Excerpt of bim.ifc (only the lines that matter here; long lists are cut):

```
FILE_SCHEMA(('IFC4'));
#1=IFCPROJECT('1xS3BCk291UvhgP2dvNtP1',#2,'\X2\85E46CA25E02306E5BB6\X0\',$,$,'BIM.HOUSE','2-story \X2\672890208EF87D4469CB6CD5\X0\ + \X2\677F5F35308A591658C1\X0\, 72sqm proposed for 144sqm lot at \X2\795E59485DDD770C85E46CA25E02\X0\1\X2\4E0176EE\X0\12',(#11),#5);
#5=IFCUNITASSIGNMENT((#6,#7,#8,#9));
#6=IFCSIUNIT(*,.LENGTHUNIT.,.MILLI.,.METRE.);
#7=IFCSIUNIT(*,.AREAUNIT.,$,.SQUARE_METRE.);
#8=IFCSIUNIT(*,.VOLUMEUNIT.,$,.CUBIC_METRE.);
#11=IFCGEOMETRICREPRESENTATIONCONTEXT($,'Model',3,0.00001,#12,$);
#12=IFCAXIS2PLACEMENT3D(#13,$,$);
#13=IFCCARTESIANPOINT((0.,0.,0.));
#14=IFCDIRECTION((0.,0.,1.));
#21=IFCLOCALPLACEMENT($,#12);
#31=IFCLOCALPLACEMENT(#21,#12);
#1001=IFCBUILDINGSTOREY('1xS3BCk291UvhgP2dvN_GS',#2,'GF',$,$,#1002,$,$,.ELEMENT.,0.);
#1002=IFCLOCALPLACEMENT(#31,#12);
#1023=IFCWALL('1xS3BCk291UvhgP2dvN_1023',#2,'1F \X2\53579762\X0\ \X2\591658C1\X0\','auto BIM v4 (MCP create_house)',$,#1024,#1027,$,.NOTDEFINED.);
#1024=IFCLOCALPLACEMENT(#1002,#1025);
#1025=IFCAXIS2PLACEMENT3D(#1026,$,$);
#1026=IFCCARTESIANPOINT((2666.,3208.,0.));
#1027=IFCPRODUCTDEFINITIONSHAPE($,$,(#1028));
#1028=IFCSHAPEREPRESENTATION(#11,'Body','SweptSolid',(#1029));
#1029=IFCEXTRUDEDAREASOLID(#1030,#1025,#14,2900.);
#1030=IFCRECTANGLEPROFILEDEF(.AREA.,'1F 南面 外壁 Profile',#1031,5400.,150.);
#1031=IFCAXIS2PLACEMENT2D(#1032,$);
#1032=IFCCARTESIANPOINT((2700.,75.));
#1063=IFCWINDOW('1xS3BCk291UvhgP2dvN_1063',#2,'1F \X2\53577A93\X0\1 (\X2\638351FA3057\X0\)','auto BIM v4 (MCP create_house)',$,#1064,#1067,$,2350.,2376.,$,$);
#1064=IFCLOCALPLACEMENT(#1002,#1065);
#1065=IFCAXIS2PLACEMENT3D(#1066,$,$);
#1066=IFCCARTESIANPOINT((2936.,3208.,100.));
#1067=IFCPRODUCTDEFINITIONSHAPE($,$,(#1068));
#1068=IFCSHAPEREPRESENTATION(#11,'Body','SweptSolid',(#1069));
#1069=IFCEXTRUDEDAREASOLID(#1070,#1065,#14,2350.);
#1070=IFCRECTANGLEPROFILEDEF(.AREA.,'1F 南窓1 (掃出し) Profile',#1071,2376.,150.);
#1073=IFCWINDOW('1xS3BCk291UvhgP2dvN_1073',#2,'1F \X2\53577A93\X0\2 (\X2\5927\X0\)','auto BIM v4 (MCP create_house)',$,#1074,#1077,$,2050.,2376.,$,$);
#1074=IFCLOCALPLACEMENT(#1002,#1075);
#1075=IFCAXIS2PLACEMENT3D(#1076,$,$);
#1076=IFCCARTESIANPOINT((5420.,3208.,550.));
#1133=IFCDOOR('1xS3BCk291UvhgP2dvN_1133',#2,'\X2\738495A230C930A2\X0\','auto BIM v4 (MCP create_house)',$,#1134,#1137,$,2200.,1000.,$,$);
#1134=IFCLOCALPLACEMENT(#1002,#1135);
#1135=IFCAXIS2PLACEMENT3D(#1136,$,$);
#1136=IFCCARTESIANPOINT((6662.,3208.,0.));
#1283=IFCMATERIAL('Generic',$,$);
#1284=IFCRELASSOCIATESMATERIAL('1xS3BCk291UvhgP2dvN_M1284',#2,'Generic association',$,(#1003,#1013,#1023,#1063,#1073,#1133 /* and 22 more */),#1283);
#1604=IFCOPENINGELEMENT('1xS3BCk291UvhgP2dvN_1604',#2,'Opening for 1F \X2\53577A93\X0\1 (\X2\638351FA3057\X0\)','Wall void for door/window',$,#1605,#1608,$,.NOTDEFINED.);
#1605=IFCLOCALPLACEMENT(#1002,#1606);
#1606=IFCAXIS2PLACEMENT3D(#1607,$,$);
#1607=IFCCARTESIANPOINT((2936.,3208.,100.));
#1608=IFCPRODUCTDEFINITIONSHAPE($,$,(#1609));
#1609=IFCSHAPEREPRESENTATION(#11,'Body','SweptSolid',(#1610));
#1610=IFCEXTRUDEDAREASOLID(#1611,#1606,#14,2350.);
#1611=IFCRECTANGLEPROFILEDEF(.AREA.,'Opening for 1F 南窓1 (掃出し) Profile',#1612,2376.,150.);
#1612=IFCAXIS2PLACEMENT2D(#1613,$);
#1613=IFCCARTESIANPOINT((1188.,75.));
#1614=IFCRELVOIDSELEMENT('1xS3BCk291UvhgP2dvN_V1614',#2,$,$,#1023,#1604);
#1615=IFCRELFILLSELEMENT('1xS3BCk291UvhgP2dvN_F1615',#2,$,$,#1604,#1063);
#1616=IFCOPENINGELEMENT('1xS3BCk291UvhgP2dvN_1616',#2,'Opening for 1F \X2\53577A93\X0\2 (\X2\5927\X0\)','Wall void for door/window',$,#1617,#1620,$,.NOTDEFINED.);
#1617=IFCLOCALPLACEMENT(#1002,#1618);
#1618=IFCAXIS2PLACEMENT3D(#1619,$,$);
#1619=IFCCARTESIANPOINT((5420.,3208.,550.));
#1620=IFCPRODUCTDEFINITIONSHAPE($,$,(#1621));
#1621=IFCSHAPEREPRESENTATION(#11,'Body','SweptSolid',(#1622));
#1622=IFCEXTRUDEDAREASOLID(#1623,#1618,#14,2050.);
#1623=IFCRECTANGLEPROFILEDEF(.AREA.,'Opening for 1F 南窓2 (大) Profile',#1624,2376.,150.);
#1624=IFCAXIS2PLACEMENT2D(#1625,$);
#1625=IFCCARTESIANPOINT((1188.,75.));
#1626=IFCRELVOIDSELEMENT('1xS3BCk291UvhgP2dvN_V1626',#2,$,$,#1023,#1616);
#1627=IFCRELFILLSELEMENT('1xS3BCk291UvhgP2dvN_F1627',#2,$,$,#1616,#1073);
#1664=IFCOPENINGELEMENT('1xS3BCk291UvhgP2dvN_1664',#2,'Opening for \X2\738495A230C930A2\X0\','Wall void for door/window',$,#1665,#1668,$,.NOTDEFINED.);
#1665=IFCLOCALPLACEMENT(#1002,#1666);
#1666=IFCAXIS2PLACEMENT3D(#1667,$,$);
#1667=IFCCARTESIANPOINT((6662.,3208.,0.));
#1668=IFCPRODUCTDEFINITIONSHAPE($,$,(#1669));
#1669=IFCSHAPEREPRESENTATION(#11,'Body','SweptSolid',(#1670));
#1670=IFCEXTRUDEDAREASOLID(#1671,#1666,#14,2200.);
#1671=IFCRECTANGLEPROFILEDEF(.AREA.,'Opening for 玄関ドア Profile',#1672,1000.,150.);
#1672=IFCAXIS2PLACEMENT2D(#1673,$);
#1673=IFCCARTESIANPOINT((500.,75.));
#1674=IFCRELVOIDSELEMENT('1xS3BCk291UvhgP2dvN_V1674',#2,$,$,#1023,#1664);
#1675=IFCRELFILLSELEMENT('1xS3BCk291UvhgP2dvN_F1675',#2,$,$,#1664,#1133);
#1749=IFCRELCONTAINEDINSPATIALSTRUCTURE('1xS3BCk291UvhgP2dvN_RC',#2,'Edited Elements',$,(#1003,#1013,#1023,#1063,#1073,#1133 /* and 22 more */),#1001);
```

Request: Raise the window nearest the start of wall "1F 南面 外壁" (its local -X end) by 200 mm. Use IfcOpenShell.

```python
import numpy as np
import ifcopenshell
import ifcopenshell.api.geometry
import ifcopenshell.util.placement
import ifcopenshell.util.unit

model = ifcopenshell.open("bim.ifc")
unit_scale = ifcopenshell.util.unit.calculate_unit_scale(model)

window = model.by_guid("1xS3BCk291UvhgP2dvN_1063")
opening = window.FillsVoids[0].RelatingOpeningElement
dz = 0.2 / unit_scale

shift = np.array([0.0, 0.0, dz])
# The window is not placed relative to its opening, so move both.
for product in (opening, window):
    matrix = ifcopenshell.util.placement.get_local_placement(product.ObjectPlacement)
    matrix[:3, 3] += shift
    ifcopenshell.api.geometry.edit_object_placement(model, product=product, matrix=matrix, is_si=False)

print(f"moved by {dz * unit_scale:+.3f} m")

model.write("bim-out.ifc")
```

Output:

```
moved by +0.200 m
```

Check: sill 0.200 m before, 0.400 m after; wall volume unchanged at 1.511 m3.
